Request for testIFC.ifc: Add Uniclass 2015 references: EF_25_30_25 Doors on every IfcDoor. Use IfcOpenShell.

First a look at what the model holds.

```python
import ifcopenshell

model = ifcopenshell.open("testIFC.ifc")
print(model.schema)
print("classifications:", [c.Name for c in model.by_type("IfcClassification")])
for ifc_class in ("IfcDoor", "IfcRoof", "IfcStair", "IfcWall", "IfcWindow"):
    print(ifc_class, len(model.by_type(ifc_class)))
```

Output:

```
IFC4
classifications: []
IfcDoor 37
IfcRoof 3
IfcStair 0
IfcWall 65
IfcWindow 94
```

```python
import ifcopenshell
import ifcopenshell.api.classification

model = ifcopenshell.open("testIFC.ifc")

system = ifcopenshell.api.classification.add_classification(model, classification="Uniclass 2015")

codes = {
    "IfcDoor": ("EF_25_30_25", "Doors"),
}
for ifc_class, (code, name) in codes.items():
    products = model.by_type(ifc_class)
    ifcopenshell.api.classification.add_reference(
        model, products=products, classification=system, identification=code, name=name
    )
    print(code, len(products))

model.write("testIFC_edited.ifc")
```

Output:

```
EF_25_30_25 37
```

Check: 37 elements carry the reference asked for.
